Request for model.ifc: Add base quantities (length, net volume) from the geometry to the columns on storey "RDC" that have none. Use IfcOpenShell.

First a look at what the model holds.

```python
import ifcopenshell
import ifcopenshell.util.element
import ifcopenshell.util.unit

model = ifcopenshell.open("model.ifc")
print(model.schema)
for unit_type in ("LENGTHUNIT", "AREAUNIT", "VOLUMEUNIT"):
    print(unit_type, ifcopenshell.util.unit.calculate_unit_scale(model, unit_type))
storey = next(s for s in model.by_type("IfcBuildingStorey") if s.Name == "RDC")
columns = [e for e in ifcopenshell.util.element.get_decomposition(storey) if e.is_a("IfcColumn")]
for e in sorted(columns, key=lambda e: e.id()):
    print(e.id(), e.is_a(), e.Name, list(ifcopenshell.util.element.get_psets(e, qtos_only=True)), sep=" | ")
```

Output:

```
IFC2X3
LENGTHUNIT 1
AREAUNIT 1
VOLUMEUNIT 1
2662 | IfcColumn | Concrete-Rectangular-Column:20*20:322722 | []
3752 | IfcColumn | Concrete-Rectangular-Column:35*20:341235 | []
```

```python
import ifcopenshell
import ifcopenshell.api.pset
import ifcopenshell.geom
import ifcopenshell.util.element
import ifcopenshell.util.shape
import ifcopenshell.util.unit

model = ifcopenshell.open("model.ifc")
unit_scale = ifcopenshell.util.unit.calculate_unit_scale(model)
volume_scale = ifcopenshell.util.unit.calculate_unit_scale(model, "VOLUMEUNIT")
settings = ifcopenshell.geom.settings()

storey = next(s for s in model.by_type("IfcBuildingStorey") if s.Name == "RDC")
columns = [e for e in ifcopenshell.util.element.get_decomposition(storey) if e.is_a("IfcColumn")]

for e in sorted(columns, key=lambda e: e.id()):
    if ifcopenshell.util.element.get_psets(e, qtos_only=True, should_inherit=False):
        continue
    # Geometry comes back in metres, in the element's own axes.
    shape = ifcopenshell.geom.create_shape(settings, e)
    values = {
        "Length": ifcopenshell.util.shape.get_z(shape.geometry) / unit_scale,
        "NetVolume": ifcopenshell.util.shape.get_volume(shape.geometry) / volume_scale,
    }
    qto = ifcopenshell.api.pset.add_qto(model, product=e, name="BaseQuantities")
    ifcopenshell.api.pset.edit_qto(model, qto=qto, properties=values)
    print(e.id(), {k: round(v, 3) for k, v in values.items()})

model.write("model_updated.ifc")
```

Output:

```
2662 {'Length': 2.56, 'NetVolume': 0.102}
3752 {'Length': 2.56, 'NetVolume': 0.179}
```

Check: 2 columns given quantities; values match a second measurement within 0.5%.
